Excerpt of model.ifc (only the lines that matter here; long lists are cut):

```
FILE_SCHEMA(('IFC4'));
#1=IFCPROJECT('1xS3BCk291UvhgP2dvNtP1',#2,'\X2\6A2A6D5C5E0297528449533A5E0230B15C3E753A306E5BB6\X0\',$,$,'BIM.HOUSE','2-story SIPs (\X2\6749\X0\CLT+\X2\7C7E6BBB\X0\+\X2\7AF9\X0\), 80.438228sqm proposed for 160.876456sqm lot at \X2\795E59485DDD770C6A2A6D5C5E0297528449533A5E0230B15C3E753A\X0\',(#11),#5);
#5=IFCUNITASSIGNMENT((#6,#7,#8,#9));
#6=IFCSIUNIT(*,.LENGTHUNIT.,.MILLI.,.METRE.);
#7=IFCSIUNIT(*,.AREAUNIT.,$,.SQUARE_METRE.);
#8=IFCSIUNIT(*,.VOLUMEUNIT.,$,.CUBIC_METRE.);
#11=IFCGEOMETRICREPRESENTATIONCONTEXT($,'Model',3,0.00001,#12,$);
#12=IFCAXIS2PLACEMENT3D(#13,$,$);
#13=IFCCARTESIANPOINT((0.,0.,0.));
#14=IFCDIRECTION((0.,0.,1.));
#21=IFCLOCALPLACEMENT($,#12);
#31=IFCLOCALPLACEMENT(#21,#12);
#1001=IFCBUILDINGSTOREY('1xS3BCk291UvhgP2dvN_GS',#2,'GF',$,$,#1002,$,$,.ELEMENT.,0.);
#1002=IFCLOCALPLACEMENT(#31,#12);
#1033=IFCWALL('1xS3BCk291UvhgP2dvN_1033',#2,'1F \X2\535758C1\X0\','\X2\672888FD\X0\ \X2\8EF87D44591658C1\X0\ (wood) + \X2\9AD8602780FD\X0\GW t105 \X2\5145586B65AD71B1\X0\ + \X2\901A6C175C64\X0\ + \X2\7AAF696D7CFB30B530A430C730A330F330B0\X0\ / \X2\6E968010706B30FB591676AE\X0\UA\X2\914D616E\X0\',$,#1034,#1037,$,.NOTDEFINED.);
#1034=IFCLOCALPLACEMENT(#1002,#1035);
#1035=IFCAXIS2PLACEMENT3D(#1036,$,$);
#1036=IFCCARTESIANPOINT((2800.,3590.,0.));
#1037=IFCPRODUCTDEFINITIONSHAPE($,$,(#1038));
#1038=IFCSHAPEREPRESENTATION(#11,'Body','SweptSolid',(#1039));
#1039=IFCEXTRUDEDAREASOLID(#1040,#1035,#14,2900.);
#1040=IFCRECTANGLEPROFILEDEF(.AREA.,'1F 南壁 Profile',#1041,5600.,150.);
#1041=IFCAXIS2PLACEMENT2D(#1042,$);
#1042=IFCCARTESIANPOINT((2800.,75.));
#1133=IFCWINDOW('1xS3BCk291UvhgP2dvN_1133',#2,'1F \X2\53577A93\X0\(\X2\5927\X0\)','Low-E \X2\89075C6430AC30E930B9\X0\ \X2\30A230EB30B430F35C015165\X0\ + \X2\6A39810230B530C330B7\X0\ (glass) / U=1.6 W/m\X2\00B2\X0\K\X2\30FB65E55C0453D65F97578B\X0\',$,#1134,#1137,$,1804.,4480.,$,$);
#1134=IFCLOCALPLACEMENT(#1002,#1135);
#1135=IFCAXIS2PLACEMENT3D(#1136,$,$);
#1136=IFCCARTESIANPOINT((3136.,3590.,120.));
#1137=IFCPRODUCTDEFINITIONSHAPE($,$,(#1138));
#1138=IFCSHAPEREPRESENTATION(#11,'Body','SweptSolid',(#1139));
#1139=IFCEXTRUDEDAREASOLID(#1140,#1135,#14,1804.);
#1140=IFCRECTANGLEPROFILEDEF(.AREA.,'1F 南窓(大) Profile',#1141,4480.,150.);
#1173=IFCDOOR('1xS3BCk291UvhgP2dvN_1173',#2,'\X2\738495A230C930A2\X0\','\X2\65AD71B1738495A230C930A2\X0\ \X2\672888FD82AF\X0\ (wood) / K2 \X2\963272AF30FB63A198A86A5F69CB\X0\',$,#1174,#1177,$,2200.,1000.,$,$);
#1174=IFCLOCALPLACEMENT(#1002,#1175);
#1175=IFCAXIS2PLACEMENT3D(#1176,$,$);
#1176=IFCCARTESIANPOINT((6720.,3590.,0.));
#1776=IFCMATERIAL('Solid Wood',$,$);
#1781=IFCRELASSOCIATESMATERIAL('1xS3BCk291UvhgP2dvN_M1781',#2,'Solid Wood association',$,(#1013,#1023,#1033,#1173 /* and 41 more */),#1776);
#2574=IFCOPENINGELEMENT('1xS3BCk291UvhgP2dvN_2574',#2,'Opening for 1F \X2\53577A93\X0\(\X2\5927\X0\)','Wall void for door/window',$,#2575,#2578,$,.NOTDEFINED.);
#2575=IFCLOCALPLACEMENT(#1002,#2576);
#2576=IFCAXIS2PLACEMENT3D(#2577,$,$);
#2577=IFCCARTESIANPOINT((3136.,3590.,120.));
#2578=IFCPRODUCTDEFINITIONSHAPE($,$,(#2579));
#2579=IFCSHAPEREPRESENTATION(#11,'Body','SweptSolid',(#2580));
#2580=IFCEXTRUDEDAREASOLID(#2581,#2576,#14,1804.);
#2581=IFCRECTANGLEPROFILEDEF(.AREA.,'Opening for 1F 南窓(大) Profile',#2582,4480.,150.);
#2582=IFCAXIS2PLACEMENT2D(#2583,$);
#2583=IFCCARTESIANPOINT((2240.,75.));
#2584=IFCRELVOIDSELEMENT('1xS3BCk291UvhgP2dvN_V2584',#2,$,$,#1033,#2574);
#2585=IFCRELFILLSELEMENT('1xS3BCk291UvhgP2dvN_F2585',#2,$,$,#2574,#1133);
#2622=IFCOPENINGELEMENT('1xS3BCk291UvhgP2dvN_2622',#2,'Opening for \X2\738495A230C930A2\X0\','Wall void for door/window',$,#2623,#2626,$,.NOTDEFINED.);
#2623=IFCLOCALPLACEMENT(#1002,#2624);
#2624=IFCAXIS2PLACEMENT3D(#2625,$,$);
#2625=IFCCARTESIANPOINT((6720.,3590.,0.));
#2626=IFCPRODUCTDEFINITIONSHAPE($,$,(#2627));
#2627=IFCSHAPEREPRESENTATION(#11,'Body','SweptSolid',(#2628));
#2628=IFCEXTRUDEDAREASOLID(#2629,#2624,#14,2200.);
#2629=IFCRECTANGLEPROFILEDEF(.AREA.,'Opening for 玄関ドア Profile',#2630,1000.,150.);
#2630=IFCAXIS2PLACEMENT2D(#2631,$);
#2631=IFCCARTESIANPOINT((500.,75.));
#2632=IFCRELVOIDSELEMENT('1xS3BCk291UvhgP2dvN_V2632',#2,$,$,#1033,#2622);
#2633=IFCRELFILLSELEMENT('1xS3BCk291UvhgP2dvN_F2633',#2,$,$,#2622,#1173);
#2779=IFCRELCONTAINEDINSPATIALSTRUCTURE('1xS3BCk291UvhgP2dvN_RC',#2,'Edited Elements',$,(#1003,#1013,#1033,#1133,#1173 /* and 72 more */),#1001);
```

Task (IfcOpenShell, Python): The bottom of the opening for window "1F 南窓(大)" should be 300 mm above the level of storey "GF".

```python
import numpy as np
import ifcopenshell
import ifcopenshell.api.geometry
import ifcopenshell.geom
import ifcopenshell.util.element
import ifcopenshell.util.placement
import ifcopenshell.util.shape
import ifcopenshell.util.unit

model = ifcopenshell.open("model.ifc")
unit_scale = ifcopenshell.util.unit.calculate_unit_scale(model)

window = model.by_guid("1xS3BCk291UvhgP2dvN_1133")
opening = window.FillsVoids[0].RelatingOpeningElement
storey = ifcopenshell.util.element.get_container(window, ifc_class="IfcBuildingStorey")
level = ifcopenshell.util.placement.get_local_placement(storey.ObjectPlacement)[2, 3]

# The opening's origin need not be at the sill, so measure its lowest point.
shape = ifcopenshell.geom.create_shape(ifcopenshell.geom.settings(), opening)
bottom = ifcopenshell.util.shape.get_shape_bottom_elevation(shape, shape.geometry) / unit_scale
dz = level + 300.0 - bottom

shift = np.array([0.0, 0.0, dz])
# The window is not placed relative to its opening, so move both.
for product in (opening, window):
    matrix = ifcopenshell.util.placement.get_local_placement(product.ObjectPlacement)
    matrix[:3, 3] += shift
    ifcopenshell.api.geometry.edit_object_placement(model, product=product, matrix=matrix, is_si=False)

print(f"moved by {dz * unit_scale:+.3f} m")

model.write("model_v2.ifc")
```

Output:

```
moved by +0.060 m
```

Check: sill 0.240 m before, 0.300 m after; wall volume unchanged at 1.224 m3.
